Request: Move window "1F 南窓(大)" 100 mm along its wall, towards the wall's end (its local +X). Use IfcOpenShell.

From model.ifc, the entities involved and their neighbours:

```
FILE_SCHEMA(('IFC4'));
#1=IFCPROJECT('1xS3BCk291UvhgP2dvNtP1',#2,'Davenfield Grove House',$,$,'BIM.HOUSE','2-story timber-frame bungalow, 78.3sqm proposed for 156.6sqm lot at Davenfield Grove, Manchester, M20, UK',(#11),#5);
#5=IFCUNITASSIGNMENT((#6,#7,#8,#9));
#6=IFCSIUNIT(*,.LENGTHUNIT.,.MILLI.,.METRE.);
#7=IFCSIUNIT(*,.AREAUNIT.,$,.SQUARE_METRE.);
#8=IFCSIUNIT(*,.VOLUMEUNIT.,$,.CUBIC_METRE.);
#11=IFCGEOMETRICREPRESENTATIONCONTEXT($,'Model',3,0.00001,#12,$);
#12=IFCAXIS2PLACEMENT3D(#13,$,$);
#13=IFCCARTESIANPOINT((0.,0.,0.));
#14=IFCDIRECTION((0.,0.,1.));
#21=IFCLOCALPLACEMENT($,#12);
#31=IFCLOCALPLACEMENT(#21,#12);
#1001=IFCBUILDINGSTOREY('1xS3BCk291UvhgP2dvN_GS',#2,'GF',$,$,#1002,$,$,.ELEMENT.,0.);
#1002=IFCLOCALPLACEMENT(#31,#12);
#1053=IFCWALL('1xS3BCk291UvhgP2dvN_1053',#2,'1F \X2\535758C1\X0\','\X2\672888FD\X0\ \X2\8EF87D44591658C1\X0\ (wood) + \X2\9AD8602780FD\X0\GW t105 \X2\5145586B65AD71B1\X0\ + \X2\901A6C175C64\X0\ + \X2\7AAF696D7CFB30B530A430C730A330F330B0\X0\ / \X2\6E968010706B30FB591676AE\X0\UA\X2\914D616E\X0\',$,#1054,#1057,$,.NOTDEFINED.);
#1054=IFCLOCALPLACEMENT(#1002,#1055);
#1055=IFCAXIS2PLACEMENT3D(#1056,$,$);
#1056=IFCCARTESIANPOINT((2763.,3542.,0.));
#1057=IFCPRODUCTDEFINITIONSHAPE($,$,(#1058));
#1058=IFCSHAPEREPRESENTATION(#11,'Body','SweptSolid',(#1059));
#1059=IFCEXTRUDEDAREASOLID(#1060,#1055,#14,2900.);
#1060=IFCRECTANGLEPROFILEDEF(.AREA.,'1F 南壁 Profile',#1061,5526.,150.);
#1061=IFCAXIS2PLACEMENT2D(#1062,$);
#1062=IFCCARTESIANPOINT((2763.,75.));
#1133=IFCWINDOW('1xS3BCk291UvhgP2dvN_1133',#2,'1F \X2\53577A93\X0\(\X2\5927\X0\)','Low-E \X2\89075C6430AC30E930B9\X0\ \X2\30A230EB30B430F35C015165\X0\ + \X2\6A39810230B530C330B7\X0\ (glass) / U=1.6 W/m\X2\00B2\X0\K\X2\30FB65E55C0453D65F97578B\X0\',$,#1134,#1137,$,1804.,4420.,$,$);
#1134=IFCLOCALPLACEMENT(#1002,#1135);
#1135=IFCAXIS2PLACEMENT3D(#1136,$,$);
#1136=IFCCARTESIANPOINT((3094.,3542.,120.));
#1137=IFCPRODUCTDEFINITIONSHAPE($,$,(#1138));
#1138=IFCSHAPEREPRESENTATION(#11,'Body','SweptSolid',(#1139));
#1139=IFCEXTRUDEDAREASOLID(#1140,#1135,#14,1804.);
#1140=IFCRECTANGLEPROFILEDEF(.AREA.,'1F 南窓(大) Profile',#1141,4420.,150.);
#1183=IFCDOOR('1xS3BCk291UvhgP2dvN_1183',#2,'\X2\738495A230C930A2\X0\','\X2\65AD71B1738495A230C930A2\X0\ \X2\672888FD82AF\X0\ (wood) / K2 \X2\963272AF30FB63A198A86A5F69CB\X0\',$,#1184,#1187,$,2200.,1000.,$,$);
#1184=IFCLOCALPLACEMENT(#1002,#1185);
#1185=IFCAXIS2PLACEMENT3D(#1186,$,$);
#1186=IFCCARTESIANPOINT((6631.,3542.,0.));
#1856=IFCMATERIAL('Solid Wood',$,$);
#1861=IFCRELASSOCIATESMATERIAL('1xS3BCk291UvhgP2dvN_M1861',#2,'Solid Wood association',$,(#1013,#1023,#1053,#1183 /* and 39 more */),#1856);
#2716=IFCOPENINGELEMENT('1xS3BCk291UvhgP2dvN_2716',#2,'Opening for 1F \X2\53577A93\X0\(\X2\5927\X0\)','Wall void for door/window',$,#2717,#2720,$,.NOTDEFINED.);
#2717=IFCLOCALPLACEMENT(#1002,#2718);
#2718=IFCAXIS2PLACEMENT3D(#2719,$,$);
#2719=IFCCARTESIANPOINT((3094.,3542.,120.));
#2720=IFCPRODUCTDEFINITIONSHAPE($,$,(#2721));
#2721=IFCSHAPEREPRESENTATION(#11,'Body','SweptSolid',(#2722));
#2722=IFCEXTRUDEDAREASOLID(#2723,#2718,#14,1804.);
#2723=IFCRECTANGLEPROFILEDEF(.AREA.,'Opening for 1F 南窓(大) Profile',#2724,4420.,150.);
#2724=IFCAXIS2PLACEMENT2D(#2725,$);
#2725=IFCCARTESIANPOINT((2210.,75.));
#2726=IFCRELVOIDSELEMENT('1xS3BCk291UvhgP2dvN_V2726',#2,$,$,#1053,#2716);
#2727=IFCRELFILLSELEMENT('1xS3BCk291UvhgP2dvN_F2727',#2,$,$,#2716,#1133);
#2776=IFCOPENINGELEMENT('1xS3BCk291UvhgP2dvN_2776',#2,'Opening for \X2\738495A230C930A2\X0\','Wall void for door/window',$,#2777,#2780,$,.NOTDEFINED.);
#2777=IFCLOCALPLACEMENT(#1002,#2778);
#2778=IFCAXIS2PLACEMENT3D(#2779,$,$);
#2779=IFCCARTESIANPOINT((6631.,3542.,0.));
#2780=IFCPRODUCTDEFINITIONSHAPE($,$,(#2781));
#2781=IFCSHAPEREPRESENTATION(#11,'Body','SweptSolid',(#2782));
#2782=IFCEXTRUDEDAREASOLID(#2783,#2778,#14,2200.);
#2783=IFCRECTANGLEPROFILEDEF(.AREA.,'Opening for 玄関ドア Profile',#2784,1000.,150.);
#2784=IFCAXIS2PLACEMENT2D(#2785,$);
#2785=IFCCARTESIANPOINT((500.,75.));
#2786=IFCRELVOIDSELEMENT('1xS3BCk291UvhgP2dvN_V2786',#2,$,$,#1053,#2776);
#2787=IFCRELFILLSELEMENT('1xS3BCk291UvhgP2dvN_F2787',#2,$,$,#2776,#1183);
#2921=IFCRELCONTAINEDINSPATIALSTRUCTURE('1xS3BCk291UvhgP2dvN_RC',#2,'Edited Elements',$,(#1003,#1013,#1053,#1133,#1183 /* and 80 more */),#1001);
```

```python
import ifcopenshell
import ifcopenshell.api.geometry
import ifcopenshell.util.placement

model = ifcopenshell.open("model.ifc")

window = model.by_guid("1xS3BCk291UvhgP2dvN_1133")
opening = window.FillsVoids[0].RelatingOpeningElement
wall = opening.VoidsElements[0].RelatingBuildingElement

wall_matrix = ifcopenshell.util.placement.get_local_placement(wall.ObjectPlacement)
shift = wall_matrix[:3, 0] * 100.0
before = ifcopenshell.util.placement.get_local_placement(window.ObjectPlacement)[:3, 3].copy()

# The window is not placed relative to its opening, so move both.
for product in (opening, window):
    matrix = ifcopenshell.util.placement.get_local_placement(product.ObjectPlacement)
    matrix[:3, 3] += shift
    ifcopenshell.api.geometry.edit_object_placement(model, product=product, matrix=matrix, is_si=False)

after = ifcopenshell.util.placement.get_local_placement(window.ObjectPlacement)[:3, 3]
print("window moved by", (after - before).round(3) + 0.0)

model.write("model_updated.ifc")
```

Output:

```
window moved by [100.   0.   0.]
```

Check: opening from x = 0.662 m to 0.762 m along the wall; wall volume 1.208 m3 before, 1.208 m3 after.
